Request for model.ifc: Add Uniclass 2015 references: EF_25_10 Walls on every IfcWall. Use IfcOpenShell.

First a look at what the model holds.

```python
import ifcopenshell

model = ifcopenshell.open("model.ifc")
print(model.schema)
print("classifications:", [c.Name for c in model.by_type("IfcClassification")])
for ifc_class in ("IfcDoor", "IfcRoof", "IfcStair", "IfcWall", "IfcWindow"):
    print(ifc_class, len(model.by_type(ifc_class)))
```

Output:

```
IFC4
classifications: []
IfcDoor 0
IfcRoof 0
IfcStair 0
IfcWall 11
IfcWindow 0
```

```python
import ifcopenshell
import ifcopenshell.api.classification

model = ifcopenshell.open("model.ifc")

system = ifcopenshell.api.classification.add_classification(model, classification="Uniclass 2015")

codes = {
    "IfcWall": ("EF_25_10", "Walls"),
}
for ifc_class, (code, name) in codes.items():
    products = model.by_type(ifc_class)
    ifcopenshell.api.classification.add_reference(
        model, products=products, classification=system, identification=code, name=name
    )
    print(code, len(products))

model.write("model_edited.ifc")
```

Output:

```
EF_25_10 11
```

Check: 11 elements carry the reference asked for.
